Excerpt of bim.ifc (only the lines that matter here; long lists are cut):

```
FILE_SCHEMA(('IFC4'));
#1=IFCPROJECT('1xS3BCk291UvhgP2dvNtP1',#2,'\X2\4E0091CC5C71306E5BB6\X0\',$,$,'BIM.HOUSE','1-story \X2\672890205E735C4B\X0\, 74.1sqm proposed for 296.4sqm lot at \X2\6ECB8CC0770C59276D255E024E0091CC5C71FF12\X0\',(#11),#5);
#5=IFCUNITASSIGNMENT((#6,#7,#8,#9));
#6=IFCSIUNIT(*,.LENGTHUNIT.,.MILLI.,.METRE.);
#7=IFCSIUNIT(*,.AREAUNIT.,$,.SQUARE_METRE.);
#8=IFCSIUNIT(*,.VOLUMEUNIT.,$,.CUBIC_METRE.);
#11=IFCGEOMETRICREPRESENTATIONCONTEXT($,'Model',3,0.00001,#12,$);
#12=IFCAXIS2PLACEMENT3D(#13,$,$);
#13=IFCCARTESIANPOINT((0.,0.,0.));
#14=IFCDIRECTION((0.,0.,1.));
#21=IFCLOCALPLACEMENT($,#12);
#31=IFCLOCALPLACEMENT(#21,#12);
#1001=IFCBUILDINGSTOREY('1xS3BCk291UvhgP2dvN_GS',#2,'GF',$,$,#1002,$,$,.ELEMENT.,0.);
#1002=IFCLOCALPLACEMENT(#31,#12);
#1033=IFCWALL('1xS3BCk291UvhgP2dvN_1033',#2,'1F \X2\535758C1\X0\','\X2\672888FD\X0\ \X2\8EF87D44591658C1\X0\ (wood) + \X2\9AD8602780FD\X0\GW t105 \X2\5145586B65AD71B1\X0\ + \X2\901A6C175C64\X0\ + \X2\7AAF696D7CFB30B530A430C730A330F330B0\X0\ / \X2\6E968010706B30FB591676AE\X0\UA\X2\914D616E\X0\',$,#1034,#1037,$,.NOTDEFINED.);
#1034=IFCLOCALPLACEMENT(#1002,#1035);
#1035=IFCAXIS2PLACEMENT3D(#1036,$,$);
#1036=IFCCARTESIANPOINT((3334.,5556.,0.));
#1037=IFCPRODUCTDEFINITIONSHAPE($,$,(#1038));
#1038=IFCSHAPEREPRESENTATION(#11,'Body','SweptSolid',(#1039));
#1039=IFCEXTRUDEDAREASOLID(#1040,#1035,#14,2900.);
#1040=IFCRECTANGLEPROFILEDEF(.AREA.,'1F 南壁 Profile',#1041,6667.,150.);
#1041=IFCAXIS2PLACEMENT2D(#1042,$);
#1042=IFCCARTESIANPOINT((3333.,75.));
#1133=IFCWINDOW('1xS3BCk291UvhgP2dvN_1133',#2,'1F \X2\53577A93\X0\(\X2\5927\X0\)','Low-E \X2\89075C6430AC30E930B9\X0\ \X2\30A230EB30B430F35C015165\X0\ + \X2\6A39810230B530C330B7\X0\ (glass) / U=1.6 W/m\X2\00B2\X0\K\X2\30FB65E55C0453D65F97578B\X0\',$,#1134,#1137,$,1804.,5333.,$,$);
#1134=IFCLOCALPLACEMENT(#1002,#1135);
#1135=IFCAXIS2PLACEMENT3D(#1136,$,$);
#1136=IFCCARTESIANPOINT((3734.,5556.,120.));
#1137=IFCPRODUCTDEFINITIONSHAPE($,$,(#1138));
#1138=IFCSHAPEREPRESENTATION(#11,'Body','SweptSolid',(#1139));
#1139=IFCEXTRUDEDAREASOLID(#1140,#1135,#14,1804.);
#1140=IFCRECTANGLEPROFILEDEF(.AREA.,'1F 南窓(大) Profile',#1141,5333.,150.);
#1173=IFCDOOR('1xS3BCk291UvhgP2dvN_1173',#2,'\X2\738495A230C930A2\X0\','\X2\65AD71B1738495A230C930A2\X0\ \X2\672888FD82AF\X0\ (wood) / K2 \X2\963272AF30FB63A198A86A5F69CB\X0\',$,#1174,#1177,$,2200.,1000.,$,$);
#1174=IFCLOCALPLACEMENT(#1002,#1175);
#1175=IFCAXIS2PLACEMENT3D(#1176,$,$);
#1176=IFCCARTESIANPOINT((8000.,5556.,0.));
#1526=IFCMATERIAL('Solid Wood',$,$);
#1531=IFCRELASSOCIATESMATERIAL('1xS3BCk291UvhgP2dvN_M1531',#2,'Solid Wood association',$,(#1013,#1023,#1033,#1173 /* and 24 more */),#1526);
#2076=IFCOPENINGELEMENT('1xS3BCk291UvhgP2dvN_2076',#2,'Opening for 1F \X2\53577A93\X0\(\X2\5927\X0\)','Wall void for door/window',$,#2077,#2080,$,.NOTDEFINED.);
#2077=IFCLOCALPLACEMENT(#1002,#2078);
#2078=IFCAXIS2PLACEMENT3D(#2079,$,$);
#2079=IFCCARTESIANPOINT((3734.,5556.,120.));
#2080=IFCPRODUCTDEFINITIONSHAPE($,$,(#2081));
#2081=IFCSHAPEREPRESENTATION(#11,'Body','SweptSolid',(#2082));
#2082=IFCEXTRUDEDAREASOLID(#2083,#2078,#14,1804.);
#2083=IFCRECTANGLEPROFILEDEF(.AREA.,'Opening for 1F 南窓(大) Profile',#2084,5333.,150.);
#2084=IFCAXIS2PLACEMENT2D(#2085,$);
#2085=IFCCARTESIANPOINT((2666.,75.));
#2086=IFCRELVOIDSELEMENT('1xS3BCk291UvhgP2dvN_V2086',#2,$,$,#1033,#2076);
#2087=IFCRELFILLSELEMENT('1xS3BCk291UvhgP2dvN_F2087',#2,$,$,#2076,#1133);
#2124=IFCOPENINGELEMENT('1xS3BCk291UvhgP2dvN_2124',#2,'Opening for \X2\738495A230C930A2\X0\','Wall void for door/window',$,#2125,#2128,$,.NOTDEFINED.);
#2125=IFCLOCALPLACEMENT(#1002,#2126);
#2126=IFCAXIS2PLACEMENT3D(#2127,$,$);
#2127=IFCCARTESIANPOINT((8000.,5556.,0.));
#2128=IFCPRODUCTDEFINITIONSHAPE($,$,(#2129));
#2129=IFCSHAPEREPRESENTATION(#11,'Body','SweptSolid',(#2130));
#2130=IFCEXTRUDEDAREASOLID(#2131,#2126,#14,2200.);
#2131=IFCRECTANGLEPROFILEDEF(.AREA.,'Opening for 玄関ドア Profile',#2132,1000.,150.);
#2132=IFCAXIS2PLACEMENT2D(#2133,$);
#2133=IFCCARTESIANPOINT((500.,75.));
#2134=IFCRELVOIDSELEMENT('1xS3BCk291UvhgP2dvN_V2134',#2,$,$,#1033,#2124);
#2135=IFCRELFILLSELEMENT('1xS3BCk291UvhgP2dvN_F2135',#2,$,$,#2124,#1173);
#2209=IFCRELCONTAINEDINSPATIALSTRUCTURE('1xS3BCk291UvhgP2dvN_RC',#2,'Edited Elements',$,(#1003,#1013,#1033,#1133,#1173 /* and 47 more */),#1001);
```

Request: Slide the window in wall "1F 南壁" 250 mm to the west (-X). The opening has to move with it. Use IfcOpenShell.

```python
import ifcopenshell
import ifcopenshell.api.geometry
import ifcopenshell.util.placement

model = ifcopenshell.open("bim.ifc")

window = model.by_guid("1xS3BCk291UvhgP2dvN_1133")
opening = window.FillsVoids[0].RelatingOpeningElement
wall = opening.VoidsElements[0].RelatingBuildingElement

wall_matrix = ifcopenshell.util.placement.get_local_placement(wall.ObjectPlacement)
shift = wall_matrix[:3, 0] * -250.0
before = ifcopenshell.util.placement.get_local_placement(window.ObjectPlacement)[:3, 3].copy()

# The window is not placed relative to its opening, so move both.
for product in (opening, window):
    matrix = ifcopenshell.util.placement.get_local_placement(product.ObjectPlacement)
    matrix[:3, 3] += shift
    ifcopenshell.api.geometry.edit_object_placement(model, product=product, matrix=matrix, is_si=False)

after = ifcopenshell.util.placement.get_local_placement(window.ObjectPlacement)[:3, 3]
print("window moved by", (after - before).round(3) + 0.0)

model.write("bim_updated.ifc")
```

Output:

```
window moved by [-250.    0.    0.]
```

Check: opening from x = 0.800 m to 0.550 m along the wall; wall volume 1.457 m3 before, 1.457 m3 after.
